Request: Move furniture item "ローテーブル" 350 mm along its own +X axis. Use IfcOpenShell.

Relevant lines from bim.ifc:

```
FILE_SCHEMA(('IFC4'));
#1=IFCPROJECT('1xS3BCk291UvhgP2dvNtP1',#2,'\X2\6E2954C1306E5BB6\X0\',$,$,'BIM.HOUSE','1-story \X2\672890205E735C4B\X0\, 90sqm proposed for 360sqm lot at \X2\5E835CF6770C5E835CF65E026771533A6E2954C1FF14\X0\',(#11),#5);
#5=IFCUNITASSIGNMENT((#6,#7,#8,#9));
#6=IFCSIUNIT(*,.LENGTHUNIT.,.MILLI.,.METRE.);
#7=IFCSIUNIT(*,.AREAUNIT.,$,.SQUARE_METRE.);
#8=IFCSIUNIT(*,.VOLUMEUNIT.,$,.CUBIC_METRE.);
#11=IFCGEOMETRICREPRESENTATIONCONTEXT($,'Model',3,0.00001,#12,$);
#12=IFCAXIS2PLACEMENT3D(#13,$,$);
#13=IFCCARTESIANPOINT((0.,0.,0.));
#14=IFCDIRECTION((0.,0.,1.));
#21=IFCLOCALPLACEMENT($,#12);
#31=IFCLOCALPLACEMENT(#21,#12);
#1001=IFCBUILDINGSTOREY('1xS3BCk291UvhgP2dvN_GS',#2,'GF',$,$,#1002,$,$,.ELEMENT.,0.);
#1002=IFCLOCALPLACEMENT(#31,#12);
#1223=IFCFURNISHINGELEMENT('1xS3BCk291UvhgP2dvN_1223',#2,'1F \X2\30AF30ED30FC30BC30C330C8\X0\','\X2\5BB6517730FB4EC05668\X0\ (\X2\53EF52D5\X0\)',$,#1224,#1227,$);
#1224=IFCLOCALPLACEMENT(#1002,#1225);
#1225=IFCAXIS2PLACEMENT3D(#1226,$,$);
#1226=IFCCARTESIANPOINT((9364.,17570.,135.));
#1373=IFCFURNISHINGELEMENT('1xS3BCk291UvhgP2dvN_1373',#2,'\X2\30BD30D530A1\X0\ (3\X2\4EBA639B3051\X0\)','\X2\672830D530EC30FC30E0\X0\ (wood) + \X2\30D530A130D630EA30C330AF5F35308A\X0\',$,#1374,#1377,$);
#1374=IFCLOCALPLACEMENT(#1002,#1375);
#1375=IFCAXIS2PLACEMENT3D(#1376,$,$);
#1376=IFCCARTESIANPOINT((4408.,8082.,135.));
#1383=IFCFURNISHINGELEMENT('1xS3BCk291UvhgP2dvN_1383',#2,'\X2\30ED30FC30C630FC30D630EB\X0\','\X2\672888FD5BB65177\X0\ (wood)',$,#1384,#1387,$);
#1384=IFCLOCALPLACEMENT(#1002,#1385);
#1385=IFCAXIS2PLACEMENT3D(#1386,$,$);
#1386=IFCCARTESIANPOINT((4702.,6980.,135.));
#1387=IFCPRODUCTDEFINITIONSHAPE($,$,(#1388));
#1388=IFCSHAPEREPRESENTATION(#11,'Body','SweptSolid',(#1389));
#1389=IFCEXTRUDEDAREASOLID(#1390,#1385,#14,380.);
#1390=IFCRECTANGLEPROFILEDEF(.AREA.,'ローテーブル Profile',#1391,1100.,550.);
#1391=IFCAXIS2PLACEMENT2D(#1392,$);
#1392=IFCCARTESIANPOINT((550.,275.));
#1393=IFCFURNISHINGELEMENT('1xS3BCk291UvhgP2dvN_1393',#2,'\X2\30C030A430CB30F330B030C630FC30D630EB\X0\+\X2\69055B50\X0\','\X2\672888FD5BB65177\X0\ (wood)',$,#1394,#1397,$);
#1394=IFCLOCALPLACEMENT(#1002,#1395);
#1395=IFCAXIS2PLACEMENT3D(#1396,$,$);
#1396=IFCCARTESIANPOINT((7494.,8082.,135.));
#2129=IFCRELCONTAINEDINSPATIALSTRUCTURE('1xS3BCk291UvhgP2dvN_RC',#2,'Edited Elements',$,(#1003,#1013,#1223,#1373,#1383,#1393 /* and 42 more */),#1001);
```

```python
import ifcopenshell
import ifcopenshell.api.geometry
import ifcopenshell.util.placement
import ifcopenshell.util.unit

model = ifcopenshell.open("bim.ifc")
unit_scale = ifcopenshell.util.unit.calculate_unit_scale(model)

item = model.by_id(1383)
matrix = ifcopenshell.util.placement.get_local_placement(item.ObjectPlacement)
matrix[:3, 3] += matrix[:3, 0] * 0.35 / unit_scale
ifcopenshell.api.geometry.edit_object_placement(model, product=item, matrix=matrix, is_si=False)

print(ifcopenshell.util.placement.get_local_placement(item.ObjectPlacement).round(3) + 0.0)

model.write("bim-out.ifc")
```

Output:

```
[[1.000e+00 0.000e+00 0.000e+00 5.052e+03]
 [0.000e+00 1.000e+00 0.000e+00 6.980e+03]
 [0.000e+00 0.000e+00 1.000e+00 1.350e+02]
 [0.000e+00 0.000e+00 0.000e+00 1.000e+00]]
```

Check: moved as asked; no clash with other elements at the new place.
